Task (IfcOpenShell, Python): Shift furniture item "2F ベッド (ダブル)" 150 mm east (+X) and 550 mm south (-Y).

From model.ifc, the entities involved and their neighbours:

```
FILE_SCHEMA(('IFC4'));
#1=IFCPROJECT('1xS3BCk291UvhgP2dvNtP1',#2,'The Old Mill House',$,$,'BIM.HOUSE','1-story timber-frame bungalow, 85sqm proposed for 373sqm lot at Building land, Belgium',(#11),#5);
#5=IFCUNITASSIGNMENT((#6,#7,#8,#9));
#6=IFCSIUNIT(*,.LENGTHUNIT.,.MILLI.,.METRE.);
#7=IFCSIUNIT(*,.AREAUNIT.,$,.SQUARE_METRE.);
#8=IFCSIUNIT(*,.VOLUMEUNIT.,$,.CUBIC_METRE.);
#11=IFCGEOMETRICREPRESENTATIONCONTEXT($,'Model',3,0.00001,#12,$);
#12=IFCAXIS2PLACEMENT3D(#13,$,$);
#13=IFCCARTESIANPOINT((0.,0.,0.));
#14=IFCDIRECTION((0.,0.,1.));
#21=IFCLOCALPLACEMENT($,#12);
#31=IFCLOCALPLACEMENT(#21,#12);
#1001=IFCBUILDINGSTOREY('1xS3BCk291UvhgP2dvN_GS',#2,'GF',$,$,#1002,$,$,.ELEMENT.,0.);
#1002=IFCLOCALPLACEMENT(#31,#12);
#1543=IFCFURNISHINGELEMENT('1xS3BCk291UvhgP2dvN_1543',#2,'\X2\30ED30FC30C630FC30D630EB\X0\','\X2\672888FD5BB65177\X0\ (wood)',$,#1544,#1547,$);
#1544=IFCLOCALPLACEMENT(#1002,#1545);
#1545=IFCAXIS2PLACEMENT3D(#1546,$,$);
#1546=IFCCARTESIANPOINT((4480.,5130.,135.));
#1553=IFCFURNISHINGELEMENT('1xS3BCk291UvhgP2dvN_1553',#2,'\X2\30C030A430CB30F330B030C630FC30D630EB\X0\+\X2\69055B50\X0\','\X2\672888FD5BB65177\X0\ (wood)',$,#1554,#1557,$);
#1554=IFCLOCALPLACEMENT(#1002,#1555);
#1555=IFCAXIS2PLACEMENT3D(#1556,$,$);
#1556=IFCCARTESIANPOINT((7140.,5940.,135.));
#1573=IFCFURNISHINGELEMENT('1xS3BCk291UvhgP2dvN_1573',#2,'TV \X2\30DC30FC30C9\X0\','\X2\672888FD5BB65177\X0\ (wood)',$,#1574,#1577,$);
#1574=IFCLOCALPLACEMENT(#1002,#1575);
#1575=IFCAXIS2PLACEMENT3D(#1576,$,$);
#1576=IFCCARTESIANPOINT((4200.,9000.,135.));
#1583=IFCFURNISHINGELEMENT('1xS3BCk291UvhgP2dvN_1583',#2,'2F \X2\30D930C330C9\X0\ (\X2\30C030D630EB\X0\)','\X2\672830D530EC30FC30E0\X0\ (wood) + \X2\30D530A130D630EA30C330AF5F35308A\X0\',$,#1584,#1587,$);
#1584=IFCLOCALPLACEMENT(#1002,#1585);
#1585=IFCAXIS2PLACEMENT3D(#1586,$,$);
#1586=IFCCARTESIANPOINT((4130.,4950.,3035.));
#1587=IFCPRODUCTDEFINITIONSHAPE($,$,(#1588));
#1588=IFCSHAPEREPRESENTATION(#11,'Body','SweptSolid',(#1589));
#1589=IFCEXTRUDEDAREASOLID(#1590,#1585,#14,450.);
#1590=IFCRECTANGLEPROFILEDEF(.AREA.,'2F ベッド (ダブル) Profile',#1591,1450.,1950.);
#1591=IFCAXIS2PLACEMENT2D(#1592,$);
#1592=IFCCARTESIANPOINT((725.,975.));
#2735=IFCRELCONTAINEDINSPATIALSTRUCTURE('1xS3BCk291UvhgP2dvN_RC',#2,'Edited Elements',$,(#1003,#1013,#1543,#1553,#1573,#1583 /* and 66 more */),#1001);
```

```python
import ifcopenshell
import ifcopenshell.api.geometry
import ifcopenshell.util.placement
import ifcopenshell.util.unit

model = ifcopenshell.open("model.ifc")
unit_scale = ifcopenshell.util.unit.calculate_unit_scale(model)

item = model.by_guid("1xS3BCk291UvhgP2dvN_1583")
matrix = ifcopenshell.util.placement.get_local_placement(item.ObjectPlacement)
matrix[0, 3] += 0.15 / unit_scale
matrix[1, 3] -= 0.55 / unit_scale
ifcopenshell.api.geometry.edit_object_placement(model, product=item, matrix=matrix, is_si=False)

print(ifcopenshell.util.placement.get_local_placement(item.ObjectPlacement).round(3) + 0.0)

model.write("model_rev.ifc")
```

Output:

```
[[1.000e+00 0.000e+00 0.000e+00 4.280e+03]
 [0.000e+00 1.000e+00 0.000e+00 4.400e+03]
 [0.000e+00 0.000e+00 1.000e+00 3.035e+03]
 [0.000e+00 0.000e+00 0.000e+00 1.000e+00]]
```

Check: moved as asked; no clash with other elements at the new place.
